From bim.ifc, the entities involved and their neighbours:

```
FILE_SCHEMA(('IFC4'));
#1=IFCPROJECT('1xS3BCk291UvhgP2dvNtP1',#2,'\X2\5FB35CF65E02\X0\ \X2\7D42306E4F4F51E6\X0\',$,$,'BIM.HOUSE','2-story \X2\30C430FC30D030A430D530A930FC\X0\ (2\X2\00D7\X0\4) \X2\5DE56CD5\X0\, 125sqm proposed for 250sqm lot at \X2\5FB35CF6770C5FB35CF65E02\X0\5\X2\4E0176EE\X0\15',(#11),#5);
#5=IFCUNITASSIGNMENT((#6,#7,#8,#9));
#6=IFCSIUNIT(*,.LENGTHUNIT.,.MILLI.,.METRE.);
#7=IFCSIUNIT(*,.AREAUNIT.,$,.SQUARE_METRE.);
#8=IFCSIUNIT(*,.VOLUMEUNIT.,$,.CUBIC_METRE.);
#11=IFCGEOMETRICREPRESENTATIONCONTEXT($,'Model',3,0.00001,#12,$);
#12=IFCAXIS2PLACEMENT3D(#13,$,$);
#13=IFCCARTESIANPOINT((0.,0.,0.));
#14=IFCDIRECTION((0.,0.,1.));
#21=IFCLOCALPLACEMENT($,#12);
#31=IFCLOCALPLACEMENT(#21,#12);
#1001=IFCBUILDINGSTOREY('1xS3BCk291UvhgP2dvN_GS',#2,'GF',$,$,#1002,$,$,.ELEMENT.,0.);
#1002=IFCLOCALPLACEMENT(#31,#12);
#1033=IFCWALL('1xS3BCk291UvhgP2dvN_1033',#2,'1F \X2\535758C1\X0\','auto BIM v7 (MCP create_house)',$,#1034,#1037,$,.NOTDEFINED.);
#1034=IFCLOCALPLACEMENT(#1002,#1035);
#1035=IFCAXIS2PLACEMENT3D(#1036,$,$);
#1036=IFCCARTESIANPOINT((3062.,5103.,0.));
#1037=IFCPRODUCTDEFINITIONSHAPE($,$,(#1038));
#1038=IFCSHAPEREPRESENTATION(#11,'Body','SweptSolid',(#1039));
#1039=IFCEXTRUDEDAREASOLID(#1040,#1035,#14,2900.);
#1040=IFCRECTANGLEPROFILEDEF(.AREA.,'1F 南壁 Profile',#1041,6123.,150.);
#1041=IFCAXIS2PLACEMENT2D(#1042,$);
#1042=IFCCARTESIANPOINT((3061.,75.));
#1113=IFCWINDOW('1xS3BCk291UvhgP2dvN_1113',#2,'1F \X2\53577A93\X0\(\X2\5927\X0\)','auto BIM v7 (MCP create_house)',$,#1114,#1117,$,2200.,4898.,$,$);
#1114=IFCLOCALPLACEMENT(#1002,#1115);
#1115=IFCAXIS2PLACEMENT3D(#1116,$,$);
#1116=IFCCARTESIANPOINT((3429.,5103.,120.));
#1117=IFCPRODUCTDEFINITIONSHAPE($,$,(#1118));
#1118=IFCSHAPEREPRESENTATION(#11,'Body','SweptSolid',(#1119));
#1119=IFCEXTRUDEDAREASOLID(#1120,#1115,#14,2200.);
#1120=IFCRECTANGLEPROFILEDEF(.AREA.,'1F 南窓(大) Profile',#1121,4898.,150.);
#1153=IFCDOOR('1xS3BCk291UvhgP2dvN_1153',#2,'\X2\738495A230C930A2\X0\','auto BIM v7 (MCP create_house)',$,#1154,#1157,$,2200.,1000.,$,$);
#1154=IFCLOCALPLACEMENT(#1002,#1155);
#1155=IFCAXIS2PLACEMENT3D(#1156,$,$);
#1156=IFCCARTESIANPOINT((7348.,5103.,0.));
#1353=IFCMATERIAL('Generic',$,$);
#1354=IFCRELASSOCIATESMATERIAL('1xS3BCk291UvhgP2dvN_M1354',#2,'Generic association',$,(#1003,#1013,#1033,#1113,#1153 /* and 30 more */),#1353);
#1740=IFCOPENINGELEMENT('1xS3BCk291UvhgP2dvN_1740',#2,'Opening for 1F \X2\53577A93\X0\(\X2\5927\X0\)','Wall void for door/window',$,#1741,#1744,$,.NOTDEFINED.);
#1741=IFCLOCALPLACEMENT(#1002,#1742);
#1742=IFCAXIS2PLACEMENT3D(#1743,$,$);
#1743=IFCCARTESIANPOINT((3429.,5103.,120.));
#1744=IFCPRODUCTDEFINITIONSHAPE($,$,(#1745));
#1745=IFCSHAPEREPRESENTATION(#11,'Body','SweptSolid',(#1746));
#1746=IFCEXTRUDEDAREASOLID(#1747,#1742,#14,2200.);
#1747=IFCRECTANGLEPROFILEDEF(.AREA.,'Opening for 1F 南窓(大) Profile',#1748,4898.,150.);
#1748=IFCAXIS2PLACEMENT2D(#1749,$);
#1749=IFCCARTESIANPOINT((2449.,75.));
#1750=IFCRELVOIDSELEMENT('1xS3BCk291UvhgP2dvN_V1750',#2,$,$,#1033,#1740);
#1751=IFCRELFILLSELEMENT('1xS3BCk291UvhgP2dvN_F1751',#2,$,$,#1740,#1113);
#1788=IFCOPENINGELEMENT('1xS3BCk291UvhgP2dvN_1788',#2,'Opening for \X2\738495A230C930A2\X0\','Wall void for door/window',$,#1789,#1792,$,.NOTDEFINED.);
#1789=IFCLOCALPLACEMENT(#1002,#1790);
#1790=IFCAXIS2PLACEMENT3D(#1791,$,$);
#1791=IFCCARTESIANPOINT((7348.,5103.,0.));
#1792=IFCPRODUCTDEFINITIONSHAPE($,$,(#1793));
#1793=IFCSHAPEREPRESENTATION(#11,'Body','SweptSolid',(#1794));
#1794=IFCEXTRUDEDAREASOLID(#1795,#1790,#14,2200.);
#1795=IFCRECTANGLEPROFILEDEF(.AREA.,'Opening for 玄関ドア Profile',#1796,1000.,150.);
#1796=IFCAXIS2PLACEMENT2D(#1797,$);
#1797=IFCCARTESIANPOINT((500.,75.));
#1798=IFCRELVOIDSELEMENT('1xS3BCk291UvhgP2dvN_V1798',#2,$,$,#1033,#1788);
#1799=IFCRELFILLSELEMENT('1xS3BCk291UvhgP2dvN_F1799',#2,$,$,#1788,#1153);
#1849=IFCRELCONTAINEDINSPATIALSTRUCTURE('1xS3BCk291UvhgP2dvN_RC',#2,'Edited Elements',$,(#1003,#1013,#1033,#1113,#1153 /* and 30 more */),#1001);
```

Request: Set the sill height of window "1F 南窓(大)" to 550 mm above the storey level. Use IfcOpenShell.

```python
import numpy as np
import ifcopenshell
import ifcopenshell.api.geometry
import ifcopenshell.geom
import ifcopenshell.util.element
import ifcopenshell.util.placement
import ifcopenshell.util.shape
import ifcopenshell.util.unit

model = ifcopenshell.open("bim.ifc")
unit_scale = ifcopenshell.util.unit.calculate_unit_scale(model)

window = model.by_guid("1xS3BCk291UvhgP2dvN_1113")
opening = window.FillsVoids[0].RelatingOpeningElement
storey = ifcopenshell.util.element.get_container(window, ifc_class="IfcBuildingStorey")
level = ifcopenshell.util.placement.get_local_placement(storey.ObjectPlacement)[2, 3]

# The opening's origin need not be at the sill, so measure its lowest point.
shape = ifcopenshell.geom.create_shape(ifcopenshell.geom.settings(), opening)
bottom = ifcopenshell.util.shape.get_shape_bottom_elevation(shape, shape.geometry) / unit_scale
dz = level + 0.55 / unit_scale - bottom

shift = np.array([0.0, 0.0, dz])
# The window is not placed relative to its opening, so move both.
for product in (opening, window):
    matrix = ifcopenshell.util.placement.get_local_placement(product.ObjectPlacement)
    matrix[:3, 3] += shift
    ifcopenshell.api.geometry.edit_object_placement(model, product=product, matrix=matrix, is_si=False)

print(f"moved by {dz * unit_scale:+.3f} m")

model.write("bim-out.ifc")
```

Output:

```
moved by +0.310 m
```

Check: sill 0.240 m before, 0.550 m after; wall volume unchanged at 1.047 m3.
